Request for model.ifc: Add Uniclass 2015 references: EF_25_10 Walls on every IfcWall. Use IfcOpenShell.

First a look at what the model holds.

```python
import ifcopenshell

model = ifcopenshell.open("model.ifc")
print(model.schema)
print("classifications:", [c.Name for c in model.by_type("IfcClassification")])
for ifc_class in ("IfcDoor", "IfcRoof", "IfcStair", "IfcWall", "IfcWindow"):
    print(ifc_class, len(model.by_type(ifc_class)))
```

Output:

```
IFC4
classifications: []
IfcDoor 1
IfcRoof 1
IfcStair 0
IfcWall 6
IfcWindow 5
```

```python
import ifcopenshell
import ifcopenshell.api.classification

model = ifcopenshell.open("model.ifc")

system = ifcopenshell.api.classification.add_classification(model, classification="Uniclass 2015")

codes = {
    "IfcWall": ("EF_25_10", "Walls"),
}
for ifc_class, (code, name) in codes.items():
    products = model.by_type(ifc_class)
    ifcopenshell.api.classification.add_reference(
        model, products=products, classification=system, identification=code, name=name
    )
    print(code, len(products))

model.write("model_v2.ifc")
```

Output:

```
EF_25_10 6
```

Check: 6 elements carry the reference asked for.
